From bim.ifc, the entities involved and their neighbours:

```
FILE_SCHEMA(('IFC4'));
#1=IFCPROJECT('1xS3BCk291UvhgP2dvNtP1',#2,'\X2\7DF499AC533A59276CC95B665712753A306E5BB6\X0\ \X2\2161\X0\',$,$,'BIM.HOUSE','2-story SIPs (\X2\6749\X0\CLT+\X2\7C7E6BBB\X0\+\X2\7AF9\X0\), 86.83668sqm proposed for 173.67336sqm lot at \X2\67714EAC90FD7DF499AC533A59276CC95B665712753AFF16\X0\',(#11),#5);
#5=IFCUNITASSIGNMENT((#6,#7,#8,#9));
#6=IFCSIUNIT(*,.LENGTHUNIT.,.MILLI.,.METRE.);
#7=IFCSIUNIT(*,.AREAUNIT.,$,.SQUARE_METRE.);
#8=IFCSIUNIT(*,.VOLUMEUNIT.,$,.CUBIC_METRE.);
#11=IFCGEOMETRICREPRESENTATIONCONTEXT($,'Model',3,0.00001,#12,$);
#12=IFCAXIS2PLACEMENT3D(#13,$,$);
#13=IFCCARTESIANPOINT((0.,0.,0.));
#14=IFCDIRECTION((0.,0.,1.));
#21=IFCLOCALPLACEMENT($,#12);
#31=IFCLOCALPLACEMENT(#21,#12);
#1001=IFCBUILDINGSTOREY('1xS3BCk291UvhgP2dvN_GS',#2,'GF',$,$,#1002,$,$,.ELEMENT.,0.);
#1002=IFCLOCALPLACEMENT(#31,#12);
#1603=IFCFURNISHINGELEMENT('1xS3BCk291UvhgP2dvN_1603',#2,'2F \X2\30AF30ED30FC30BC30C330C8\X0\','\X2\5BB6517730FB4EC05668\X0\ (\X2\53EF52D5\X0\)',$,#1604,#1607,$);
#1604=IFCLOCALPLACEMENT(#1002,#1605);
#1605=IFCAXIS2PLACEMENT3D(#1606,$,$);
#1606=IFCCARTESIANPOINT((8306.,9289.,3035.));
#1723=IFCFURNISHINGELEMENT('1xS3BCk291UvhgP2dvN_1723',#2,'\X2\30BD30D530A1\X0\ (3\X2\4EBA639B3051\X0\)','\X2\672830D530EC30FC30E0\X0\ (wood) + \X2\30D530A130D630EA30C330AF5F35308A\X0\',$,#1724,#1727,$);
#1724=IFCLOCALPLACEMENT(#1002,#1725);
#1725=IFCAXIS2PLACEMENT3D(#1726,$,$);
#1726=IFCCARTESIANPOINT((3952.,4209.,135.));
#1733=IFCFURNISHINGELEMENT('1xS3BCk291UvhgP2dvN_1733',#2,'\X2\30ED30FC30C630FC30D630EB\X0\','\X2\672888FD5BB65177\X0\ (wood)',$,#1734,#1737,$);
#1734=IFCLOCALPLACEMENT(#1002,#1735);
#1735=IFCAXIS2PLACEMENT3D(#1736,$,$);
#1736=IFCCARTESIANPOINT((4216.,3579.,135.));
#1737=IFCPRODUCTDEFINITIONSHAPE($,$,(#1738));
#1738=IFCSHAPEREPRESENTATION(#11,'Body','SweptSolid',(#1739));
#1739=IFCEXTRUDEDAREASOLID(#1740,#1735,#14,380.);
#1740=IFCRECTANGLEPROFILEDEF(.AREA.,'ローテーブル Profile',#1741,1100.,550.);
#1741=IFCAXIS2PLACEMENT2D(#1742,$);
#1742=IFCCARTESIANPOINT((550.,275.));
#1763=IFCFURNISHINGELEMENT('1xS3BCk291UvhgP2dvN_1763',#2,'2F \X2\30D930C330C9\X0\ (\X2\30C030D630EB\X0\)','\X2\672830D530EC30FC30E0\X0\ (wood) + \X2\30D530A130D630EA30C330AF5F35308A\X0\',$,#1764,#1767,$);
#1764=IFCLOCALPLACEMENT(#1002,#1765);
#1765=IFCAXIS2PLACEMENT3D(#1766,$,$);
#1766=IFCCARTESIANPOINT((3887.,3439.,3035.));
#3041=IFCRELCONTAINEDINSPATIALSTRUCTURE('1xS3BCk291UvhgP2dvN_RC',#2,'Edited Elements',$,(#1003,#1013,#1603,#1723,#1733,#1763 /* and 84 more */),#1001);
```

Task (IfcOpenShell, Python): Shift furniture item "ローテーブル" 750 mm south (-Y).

```python
import ifcopenshell
import ifcopenshell.api.geometry
import ifcopenshell.util.placement

model = ifcopenshell.open("bim.ifc")

item = model.by_guid("1xS3BCk291UvhgP2dvN_1733")
matrix = ifcopenshell.util.placement.get_local_placement(item.ObjectPlacement)
matrix[1, 3] -= 750.0
ifcopenshell.api.geometry.edit_object_placement(model, product=item, matrix=matrix, is_si=False)

print(ifcopenshell.util.placement.get_local_placement(item.ObjectPlacement).round(3) + 0.0)

model.write("bim_v2.ifc")
```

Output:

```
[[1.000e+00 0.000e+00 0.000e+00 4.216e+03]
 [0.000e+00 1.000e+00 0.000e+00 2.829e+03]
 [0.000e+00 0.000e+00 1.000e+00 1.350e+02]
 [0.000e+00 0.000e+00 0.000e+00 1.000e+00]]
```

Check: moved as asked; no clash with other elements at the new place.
